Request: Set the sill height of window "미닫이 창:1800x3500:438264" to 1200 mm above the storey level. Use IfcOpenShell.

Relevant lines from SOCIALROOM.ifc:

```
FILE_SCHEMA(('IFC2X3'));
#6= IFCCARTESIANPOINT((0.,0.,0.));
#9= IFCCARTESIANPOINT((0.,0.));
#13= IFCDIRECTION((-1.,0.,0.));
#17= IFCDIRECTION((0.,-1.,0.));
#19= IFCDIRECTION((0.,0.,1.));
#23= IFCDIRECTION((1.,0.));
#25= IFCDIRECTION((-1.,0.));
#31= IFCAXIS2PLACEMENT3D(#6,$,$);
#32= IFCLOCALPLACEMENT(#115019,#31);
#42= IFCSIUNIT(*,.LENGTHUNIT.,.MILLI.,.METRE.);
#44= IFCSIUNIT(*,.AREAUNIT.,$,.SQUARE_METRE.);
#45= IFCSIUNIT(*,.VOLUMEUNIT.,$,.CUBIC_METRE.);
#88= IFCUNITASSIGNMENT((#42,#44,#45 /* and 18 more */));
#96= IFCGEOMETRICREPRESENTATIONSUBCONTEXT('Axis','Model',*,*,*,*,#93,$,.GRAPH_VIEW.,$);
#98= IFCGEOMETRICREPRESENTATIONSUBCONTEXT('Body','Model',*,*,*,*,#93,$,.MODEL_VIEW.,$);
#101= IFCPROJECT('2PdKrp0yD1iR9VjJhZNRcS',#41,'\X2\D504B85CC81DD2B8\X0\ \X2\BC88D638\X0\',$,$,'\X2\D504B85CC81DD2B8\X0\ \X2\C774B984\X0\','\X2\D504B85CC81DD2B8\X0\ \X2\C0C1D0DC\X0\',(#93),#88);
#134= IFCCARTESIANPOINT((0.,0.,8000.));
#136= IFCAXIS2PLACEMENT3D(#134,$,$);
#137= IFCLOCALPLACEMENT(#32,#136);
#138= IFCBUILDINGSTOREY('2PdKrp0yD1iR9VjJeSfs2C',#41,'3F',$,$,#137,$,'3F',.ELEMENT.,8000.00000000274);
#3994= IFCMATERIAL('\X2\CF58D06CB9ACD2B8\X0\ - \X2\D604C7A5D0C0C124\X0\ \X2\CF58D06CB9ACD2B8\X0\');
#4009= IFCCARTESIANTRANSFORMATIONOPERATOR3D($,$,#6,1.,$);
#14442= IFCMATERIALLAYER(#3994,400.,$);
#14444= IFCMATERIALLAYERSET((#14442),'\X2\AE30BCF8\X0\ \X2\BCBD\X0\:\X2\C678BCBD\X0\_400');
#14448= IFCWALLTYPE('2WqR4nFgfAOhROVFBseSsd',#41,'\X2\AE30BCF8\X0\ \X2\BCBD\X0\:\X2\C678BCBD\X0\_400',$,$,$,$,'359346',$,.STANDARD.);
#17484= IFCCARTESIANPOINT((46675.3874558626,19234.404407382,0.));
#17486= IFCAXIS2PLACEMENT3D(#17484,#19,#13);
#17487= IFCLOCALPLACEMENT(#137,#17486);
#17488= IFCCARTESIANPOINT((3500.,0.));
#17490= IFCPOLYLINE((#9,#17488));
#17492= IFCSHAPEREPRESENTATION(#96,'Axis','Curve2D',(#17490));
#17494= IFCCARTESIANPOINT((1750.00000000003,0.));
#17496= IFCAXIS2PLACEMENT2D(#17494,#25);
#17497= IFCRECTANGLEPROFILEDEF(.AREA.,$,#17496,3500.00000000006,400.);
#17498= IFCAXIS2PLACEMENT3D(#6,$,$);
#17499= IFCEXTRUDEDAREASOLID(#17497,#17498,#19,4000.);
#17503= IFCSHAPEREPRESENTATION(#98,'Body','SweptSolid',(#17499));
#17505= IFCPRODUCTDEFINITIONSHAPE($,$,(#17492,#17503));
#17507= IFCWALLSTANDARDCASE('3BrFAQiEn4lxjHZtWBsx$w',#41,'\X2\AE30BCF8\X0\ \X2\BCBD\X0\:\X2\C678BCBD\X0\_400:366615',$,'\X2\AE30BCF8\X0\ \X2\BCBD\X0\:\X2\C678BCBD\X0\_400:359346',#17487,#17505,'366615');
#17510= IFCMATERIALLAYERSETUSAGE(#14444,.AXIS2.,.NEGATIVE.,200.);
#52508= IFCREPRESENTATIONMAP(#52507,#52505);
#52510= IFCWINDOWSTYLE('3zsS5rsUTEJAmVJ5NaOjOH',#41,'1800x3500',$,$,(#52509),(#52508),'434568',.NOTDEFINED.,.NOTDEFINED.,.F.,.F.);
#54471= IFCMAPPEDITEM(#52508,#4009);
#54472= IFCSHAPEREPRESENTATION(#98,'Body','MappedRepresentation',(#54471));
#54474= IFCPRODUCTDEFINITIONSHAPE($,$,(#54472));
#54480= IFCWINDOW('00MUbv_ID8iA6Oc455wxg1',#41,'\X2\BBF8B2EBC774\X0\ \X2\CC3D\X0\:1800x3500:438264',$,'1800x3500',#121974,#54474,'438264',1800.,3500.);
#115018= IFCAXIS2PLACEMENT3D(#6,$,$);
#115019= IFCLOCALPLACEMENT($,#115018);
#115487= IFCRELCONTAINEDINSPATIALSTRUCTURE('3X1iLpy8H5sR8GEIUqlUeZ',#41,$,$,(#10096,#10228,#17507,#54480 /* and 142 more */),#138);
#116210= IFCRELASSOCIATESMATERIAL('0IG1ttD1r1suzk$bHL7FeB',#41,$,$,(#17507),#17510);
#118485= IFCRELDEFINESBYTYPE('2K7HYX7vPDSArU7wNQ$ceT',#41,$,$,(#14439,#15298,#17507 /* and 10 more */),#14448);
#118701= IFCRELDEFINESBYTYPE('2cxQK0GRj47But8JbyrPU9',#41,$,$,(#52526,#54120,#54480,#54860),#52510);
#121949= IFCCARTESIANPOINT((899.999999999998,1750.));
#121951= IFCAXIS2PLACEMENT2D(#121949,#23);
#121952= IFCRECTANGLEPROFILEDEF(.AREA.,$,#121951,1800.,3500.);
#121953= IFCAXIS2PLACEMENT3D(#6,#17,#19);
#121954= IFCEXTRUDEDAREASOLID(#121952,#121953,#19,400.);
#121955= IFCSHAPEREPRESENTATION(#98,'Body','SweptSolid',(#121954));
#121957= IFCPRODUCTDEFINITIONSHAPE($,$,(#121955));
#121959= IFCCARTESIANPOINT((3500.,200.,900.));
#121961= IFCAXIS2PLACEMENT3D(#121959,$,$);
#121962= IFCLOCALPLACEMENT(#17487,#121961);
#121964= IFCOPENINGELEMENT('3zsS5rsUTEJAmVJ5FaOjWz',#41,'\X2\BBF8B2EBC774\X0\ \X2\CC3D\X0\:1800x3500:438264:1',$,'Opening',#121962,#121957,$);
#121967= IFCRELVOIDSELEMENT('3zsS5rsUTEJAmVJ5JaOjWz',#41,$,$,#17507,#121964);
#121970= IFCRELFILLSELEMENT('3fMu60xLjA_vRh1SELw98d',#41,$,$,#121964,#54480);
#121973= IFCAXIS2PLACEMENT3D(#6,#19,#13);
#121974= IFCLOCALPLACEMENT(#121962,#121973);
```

```python
import numpy as np
import ifcopenshell
import ifcopenshell.api.geometry
import ifcopenshell.geom
import ifcopenshell.util.element
import ifcopenshell.util.placement
import ifcopenshell.util.shape
import ifcopenshell.util.unit

model = ifcopenshell.open("SOCIALROOM.ifc")
unit_scale = ifcopenshell.util.unit.calculate_unit_scale(model)

window = model.by_guid("00MUbv_ID8iA6Oc455wxg1")
opening = window.FillsVoids[0].RelatingOpeningElement
storey = ifcopenshell.util.element.get_container(window, ifc_class="IfcBuildingStorey")
level = ifcopenshell.util.placement.get_local_placement(storey.ObjectPlacement)[2, 3]

# The opening's origin need not be at the sill, so measure its lowest point.
shape = ifcopenshell.geom.create_shape(ifcopenshell.geom.settings(), opening)
bottom = ifcopenshell.util.shape.get_shape_bottom_elevation(shape, shape.geometry) / unit_scale
dz = level + 1.2 / unit_scale - bottom

shift = np.array([0.0, 0.0, dz])
# The window is placed relative to its opening, so it follows when the opening moves.
matrix = ifcopenshell.util.placement.get_local_placement(opening.ObjectPlacement)
matrix[:3, 3] += shift
ifcopenshell.api.geometry.edit_object_placement(
    model, product=opening, matrix=matrix, is_si=False, should_transform_children=True
)

print(f"moved by {dz * unit_scale:+.3f} m")

model.write("SOCIALROOM_v2.ifc")
```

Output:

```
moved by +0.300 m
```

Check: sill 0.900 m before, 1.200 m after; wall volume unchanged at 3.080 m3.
